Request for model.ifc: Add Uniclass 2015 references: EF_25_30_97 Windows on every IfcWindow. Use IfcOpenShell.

First a look at what the model holds.

```python
import ifcopenshell

model = ifcopenshell.open("model.ifc")
print(model.schema)
print("classifications:", [c.Name for c in model.by_type("IfcClassification")])
for ifc_class in ("IfcDoor", "IfcRoof", "IfcStair", "IfcWall", "IfcWindow"):
    print(ifc_class, len(model.by_type(ifc_class)))
```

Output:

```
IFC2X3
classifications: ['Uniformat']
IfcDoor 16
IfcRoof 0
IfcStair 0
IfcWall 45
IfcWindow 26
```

```python
import ifcopenshell
import ifcopenshell.api.classification

model = ifcopenshell.open("model.ifc")

# IFC2X3 requires Source and Edition and has no link from the project to the system.
system = model.create_entity("IfcClassification", Source="NBS", Edition="2015", Name="Uniclass 2015")

codes = {
    "IfcWindow": ("EF_25_30_97", "Windows"),
}
for ifc_class, (code, name) in codes.items():
    products = model.by_type(ifc_class)
    ifcopenshell.api.classification.add_reference(
        model, products=products, classification=system, identification=code, name=name
    )
    print(code, len(products))

model.write("model_v2.ifc")
```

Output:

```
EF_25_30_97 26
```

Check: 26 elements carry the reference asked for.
